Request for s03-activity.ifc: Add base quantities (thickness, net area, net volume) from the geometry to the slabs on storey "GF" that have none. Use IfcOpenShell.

First a look at what the model holds.

```python
import ifcopenshell
import ifcopenshell.util.element
import ifcopenshell.util.unit

model = ifcopenshell.open("s03-activity.ifc")
print(model.schema)
for unit_type in ("LENGTHUNIT", "AREAUNIT", "VOLUMEUNIT"):
    print(unit_type, ifcopenshell.util.unit.calculate_unit_scale(model, unit_type))
storey = next(s for s in model.by_type("IfcBuildingStorey") if s.Name == "GF")
slabs = [e for e in ifcopenshell.util.element.get_decomposition(storey) if e.is_a("IfcSlab")]
for e in sorted(slabs, key=lambda e: e.id()):
    print(e.id(), e.is_a(), e.Name, list(ifcopenshell.util.element.get_psets(e, qtos_only=True)), sep=" | ")
```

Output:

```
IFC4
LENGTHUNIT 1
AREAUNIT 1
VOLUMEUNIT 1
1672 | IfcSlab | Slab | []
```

```python
import ifcopenshell
import ifcopenshell.api.pset
import ifcopenshell.geom
import ifcopenshell.util.element
import ifcopenshell.util.shape
import ifcopenshell.util.unit

model = ifcopenshell.open("s03-activity.ifc")
unit_scale = ifcopenshell.util.unit.calculate_unit_scale(model)
area_scale = ifcopenshell.util.unit.calculate_unit_scale(model, "AREAUNIT")
volume_scale = ifcopenshell.util.unit.calculate_unit_scale(model, "VOLUMEUNIT")
settings = ifcopenshell.geom.settings()

storey = next(s for s in model.by_type("IfcBuildingStorey") if s.Name == "GF")
slabs = [e for e in ifcopenshell.util.element.get_decomposition(storey) if e.is_a("IfcSlab")]

for e in sorted(slabs, key=lambda e: e.id()):
    if ifcopenshell.util.element.get_psets(e, qtos_only=True, should_inherit=False):
        continue
    # Geometry comes back in metres, in the element's own axes.
    shape = ifcopenshell.geom.create_shape(settings, e)
    values = {
        "Width": ifcopenshell.util.shape.get_z(shape.geometry) / unit_scale,
        "NetArea": ifcopenshell.util.shape.get_footprint_area(shape.geometry) / area_scale,
        "NetVolume": ifcopenshell.util.shape.get_volume(shape.geometry) / volume_scale,
    }
    qto = ifcopenshell.api.pset.add_qto(model, product=e, name="Qto_SlabBaseQuantities")
    ifcopenshell.api.pset.edit_qto(model, qto=qto, properties=values)
    print(e.id(), {k: round(v, 3) for k, v in values.items()})

model.write("s03-activity_edited.ifc")
```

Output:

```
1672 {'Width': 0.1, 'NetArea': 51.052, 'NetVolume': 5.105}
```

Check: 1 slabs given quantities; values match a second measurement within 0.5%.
